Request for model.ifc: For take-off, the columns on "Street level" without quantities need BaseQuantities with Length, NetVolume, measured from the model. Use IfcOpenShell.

First a look at what the model holds.

```python
import ifcopenshell
import ifcopenshell.util.element
import ifcopenshell.util.unit

model = ifcopenshell.open("model.ifc")
print(model.schema)
for unit_type in ("LENGTHUNIT", "AREAUNIT", "VOLUMEUNIT"):
    print(unit_type, ifcopenshell.util.unit.calculate_unit_scale(model, unit_type))
storey = next(s for s in model.by_type("IfcBuildingStorey") if s.Name == "Street level")
columns = [e for e in ifcopenshell.util.element.get_decomposition(storey) if e.is_a("IfcColumn")]
for e in sorted(columns, key=lambda e: e.id()):
    print(e.id(), e.is_a(), e.Name, list(ifcopenshell.util.element.get_psets(e, qtos_only=True)), sep=" | ")
```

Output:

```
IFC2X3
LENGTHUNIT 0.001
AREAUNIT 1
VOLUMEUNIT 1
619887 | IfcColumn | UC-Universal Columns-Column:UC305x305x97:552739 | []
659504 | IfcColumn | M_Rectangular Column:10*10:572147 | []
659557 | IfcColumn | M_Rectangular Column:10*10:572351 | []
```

```python
import ifcopenshell
import ifcopenshell.api.pset
import ifcopenshell.geom
import ifcopenshell.util.element
import ifcopenshell.util.shape
import ifcopenshell.util.unit

model = ifcopenshell.open("model.ifc")
unit_scale = ifcopenshell.util.unit.calculate_unit_scale(model)
volume_scale = ifcopenshell.util.unit.calculate_unit_scale(model, "VOLUMEUNIT")
settings = ifcopenshell.geom.settings()

storey = next(s for s in model.by_type("IfcBuildingStorey") if s.Name == "Street level")
columns = [e for e in ifcopenshell.util.element.get_decomposition(storey) if e.is_a("IfcColumn")]

for e in sorted(columns, key=lambda e: e.id()):
    if ifcopenshell.util.element.get_psets(e, qtos_only=True, should_inherit=False):
        continue
    # Geometry comes back in metres, in the element's own axes.
    shape = ifcopenshell.geom.create_shape(settings, e)
    values = {
        "Length": ifcopenshell.util.shape.get_z(shape.geometry) / unit_scale,
        "NetVolume": ifcopenshell.util.shape.get_volume(shape.geometry) / volume_scale,
    }
    qto = ifcopenshell.api.pset.add_qto(model, product=e, name="BaseQuantities")
    ifcopenshell.api.pset.edit_qto(model, qto=qto, properties=values)
    print(e.id(), {k: round(v, 3) for k, v in values.items()})

model.write("model_edited.ifc")
```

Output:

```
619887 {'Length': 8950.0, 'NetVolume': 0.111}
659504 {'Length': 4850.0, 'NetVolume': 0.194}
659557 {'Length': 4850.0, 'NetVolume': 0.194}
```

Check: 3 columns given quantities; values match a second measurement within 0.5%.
